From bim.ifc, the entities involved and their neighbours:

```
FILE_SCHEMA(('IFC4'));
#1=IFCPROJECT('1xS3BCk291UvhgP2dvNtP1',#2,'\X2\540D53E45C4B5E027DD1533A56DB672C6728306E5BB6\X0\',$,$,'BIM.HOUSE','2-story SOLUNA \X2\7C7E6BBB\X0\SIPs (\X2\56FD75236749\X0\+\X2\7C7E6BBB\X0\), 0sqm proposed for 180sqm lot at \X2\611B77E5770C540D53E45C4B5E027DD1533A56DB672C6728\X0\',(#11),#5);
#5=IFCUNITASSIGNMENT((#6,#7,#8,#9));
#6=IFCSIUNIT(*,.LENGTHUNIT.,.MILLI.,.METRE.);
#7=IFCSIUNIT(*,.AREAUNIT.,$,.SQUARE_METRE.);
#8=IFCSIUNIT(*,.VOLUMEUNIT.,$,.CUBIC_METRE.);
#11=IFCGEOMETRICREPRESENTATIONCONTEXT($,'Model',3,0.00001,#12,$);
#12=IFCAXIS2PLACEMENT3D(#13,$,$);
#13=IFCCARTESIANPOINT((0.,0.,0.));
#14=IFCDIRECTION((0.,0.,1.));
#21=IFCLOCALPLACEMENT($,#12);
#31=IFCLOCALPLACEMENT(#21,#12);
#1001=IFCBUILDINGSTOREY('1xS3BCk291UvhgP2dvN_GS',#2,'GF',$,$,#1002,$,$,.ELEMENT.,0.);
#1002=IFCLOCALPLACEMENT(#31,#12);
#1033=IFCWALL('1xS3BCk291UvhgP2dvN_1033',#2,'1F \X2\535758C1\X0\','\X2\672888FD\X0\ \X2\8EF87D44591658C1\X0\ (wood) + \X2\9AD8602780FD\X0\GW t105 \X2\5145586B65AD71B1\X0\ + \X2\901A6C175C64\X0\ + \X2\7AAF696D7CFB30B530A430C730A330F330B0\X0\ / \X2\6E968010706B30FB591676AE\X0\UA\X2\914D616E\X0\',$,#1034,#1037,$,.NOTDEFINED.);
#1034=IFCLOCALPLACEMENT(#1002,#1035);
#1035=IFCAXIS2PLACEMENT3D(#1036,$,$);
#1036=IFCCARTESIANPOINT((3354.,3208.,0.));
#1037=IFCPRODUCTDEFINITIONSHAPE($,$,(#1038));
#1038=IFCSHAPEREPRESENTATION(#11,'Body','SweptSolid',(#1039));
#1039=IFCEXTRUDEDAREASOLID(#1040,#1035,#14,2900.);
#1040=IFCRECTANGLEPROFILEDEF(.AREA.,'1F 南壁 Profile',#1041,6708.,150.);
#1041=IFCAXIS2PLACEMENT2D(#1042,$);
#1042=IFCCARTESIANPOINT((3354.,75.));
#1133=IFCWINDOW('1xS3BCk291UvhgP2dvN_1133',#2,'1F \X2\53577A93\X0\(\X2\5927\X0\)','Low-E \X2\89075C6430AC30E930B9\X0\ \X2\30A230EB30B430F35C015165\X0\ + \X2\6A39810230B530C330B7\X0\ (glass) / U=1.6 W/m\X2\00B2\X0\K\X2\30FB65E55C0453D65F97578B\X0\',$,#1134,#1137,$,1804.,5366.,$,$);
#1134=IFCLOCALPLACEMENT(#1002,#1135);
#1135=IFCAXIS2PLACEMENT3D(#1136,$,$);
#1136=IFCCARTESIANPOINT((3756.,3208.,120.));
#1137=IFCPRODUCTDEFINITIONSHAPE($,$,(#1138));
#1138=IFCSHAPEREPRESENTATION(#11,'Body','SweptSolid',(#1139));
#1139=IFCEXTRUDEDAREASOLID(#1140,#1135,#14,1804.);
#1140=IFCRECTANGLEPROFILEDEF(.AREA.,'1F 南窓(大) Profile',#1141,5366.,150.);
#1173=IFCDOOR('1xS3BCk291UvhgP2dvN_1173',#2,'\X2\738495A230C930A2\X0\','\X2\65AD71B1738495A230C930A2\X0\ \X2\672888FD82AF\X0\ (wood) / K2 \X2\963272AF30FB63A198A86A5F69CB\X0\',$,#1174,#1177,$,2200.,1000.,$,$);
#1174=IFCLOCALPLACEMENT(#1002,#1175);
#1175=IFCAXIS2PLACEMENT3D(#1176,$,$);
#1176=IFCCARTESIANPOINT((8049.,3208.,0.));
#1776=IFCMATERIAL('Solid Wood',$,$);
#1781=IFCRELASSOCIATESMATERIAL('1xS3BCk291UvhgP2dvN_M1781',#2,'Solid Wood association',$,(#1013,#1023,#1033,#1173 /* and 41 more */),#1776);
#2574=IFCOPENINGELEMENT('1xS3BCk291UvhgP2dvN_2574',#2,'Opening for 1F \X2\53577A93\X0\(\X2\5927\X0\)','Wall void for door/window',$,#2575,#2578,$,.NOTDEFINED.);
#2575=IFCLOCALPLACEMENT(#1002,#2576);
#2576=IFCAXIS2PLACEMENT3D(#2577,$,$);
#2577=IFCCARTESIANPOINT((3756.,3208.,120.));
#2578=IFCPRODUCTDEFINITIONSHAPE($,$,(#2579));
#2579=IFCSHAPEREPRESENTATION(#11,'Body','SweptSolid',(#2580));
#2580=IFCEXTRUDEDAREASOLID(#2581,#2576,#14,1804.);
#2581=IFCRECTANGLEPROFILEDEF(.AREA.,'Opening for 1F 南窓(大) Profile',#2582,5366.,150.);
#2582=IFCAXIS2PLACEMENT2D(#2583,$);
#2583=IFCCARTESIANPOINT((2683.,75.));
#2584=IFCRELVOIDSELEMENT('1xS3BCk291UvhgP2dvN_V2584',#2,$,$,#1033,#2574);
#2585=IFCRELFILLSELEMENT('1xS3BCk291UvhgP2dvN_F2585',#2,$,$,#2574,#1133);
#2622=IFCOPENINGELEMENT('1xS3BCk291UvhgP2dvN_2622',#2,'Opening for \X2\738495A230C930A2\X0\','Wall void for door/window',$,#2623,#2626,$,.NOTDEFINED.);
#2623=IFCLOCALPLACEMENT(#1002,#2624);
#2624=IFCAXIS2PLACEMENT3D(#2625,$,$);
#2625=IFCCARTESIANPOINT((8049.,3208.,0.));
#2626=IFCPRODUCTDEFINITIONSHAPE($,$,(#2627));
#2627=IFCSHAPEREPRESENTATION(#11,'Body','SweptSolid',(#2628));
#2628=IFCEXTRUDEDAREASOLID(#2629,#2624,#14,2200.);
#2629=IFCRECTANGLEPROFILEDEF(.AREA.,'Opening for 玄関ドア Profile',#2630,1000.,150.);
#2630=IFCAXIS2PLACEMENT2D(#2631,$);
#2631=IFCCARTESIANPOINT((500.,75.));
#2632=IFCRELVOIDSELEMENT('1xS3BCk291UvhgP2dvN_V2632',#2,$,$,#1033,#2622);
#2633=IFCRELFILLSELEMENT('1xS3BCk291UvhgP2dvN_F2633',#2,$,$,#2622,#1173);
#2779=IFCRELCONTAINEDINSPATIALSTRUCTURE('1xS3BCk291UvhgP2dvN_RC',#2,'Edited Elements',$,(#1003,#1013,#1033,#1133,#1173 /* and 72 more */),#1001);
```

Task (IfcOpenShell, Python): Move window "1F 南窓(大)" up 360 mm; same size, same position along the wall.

```python
import numpy as np
import ifcopenshell
import ifcopenshell.api.geometry
import ifcopenshell.util.placement
import ifcopenshell.util.unit

model = ifcopenshell.open("bim.ifc")
unit_scale = ifcopenshell.util.unit.calculate_unit_scale(model)

window = model.by_id(1133)
opening = window.FillsVoids[0].RelatingOpeningElement
dz = 360.0

shift = np.array([0.0, 0.0, dz])
# The window is not placed relative to its opening, so move both.
for product in (opening, window):
    matrix = ifcopenshell.util.placement.get_local_placement(product.ObjectPlacement)
    matrix[:3, 3] += shift
    ifcopenshell.api.geometry.edit_object_placement(model, product=product, matrix=matrix, is_si=False)

print(f"moved by {dz * unit_scale:+.3f} m")

model.write("bim-out.ifc")
```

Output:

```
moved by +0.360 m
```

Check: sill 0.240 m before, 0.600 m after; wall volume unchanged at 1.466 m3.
